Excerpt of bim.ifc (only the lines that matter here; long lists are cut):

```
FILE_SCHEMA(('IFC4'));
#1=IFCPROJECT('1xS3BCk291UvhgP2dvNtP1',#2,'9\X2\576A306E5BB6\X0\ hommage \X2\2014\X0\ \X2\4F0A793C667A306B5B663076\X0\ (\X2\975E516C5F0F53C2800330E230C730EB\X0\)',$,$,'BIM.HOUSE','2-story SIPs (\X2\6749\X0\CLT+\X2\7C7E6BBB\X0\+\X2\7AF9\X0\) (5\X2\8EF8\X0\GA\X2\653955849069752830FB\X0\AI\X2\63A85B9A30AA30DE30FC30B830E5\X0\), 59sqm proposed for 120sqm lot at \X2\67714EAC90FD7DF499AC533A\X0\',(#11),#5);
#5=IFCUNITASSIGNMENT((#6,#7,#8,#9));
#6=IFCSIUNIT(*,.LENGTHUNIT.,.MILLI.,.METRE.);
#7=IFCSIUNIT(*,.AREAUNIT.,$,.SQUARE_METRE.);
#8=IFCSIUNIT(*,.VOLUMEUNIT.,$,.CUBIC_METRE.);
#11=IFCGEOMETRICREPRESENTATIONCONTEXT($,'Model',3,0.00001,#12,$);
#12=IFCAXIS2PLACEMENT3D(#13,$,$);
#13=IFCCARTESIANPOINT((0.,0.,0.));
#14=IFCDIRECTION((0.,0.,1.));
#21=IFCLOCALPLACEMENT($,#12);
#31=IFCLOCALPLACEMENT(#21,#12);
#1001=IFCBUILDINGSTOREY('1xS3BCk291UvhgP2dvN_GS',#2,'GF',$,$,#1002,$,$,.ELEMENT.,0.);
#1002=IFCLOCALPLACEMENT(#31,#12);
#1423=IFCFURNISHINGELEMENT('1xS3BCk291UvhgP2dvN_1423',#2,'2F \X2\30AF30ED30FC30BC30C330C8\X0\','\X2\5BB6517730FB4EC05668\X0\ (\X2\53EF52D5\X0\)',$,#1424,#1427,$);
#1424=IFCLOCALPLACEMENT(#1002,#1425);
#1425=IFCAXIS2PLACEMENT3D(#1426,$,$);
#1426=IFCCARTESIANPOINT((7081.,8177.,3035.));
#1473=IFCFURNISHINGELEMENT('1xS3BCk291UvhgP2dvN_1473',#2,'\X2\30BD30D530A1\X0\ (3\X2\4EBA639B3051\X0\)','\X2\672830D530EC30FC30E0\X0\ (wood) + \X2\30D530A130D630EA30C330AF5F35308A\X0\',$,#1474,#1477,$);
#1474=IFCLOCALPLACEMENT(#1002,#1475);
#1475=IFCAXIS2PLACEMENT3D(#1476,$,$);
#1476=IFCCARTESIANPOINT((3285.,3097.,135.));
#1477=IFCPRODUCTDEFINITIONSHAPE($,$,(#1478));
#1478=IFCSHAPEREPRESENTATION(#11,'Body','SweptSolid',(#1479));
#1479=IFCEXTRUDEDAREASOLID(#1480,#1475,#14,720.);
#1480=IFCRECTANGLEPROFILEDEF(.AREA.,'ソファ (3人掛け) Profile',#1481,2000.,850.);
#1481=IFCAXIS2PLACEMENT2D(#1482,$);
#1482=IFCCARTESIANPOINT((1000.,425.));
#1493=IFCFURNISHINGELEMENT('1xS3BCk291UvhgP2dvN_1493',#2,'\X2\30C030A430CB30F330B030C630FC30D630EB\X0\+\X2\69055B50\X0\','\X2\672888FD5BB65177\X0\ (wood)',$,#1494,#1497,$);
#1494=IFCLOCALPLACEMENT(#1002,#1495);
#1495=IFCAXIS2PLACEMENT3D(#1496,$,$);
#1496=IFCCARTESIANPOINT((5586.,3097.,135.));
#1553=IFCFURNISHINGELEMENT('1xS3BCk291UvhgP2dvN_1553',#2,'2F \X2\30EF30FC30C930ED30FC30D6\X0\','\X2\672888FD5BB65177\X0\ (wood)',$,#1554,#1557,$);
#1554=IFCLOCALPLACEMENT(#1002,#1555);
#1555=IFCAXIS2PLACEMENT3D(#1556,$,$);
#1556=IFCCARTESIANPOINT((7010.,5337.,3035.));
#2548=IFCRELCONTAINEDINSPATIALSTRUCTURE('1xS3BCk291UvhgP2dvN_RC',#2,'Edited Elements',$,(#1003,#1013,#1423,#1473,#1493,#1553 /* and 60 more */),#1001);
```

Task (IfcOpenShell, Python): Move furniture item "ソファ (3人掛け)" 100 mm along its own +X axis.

```python
import ifcopenshell
import ifcopenshell.api.geometry
import ifcopenshell.util.placement
import ifcopenshell.util.unit

model = ifcopenshell.open("bim.ifc")
unit_scale = ifcopenshell.util.unit.calculate_unit_scale(model)

item = model.by_guid("1xS3BCk291UvhgP2dvN_1473")
matrix = ifcopenshell.util.placement.get_local_placement(item.ObjectPlacement)
matrix[:3, 3] += matrix[:3, 0] * 0.1 / unit_scale
ifcopenshell.api.geometry.edit_object_placement(model, product=item, matrix=matrix, is_si=False)

print(ifcopenshell.util.placement.get_local_placement(item.ObjectPlacement).round(3) + 0.0)

model.write("bim_edited.ifc")
```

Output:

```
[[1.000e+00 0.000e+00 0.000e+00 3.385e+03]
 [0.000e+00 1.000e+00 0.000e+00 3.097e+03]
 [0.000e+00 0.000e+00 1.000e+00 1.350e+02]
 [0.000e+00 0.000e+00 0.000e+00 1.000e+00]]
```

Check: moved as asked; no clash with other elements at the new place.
